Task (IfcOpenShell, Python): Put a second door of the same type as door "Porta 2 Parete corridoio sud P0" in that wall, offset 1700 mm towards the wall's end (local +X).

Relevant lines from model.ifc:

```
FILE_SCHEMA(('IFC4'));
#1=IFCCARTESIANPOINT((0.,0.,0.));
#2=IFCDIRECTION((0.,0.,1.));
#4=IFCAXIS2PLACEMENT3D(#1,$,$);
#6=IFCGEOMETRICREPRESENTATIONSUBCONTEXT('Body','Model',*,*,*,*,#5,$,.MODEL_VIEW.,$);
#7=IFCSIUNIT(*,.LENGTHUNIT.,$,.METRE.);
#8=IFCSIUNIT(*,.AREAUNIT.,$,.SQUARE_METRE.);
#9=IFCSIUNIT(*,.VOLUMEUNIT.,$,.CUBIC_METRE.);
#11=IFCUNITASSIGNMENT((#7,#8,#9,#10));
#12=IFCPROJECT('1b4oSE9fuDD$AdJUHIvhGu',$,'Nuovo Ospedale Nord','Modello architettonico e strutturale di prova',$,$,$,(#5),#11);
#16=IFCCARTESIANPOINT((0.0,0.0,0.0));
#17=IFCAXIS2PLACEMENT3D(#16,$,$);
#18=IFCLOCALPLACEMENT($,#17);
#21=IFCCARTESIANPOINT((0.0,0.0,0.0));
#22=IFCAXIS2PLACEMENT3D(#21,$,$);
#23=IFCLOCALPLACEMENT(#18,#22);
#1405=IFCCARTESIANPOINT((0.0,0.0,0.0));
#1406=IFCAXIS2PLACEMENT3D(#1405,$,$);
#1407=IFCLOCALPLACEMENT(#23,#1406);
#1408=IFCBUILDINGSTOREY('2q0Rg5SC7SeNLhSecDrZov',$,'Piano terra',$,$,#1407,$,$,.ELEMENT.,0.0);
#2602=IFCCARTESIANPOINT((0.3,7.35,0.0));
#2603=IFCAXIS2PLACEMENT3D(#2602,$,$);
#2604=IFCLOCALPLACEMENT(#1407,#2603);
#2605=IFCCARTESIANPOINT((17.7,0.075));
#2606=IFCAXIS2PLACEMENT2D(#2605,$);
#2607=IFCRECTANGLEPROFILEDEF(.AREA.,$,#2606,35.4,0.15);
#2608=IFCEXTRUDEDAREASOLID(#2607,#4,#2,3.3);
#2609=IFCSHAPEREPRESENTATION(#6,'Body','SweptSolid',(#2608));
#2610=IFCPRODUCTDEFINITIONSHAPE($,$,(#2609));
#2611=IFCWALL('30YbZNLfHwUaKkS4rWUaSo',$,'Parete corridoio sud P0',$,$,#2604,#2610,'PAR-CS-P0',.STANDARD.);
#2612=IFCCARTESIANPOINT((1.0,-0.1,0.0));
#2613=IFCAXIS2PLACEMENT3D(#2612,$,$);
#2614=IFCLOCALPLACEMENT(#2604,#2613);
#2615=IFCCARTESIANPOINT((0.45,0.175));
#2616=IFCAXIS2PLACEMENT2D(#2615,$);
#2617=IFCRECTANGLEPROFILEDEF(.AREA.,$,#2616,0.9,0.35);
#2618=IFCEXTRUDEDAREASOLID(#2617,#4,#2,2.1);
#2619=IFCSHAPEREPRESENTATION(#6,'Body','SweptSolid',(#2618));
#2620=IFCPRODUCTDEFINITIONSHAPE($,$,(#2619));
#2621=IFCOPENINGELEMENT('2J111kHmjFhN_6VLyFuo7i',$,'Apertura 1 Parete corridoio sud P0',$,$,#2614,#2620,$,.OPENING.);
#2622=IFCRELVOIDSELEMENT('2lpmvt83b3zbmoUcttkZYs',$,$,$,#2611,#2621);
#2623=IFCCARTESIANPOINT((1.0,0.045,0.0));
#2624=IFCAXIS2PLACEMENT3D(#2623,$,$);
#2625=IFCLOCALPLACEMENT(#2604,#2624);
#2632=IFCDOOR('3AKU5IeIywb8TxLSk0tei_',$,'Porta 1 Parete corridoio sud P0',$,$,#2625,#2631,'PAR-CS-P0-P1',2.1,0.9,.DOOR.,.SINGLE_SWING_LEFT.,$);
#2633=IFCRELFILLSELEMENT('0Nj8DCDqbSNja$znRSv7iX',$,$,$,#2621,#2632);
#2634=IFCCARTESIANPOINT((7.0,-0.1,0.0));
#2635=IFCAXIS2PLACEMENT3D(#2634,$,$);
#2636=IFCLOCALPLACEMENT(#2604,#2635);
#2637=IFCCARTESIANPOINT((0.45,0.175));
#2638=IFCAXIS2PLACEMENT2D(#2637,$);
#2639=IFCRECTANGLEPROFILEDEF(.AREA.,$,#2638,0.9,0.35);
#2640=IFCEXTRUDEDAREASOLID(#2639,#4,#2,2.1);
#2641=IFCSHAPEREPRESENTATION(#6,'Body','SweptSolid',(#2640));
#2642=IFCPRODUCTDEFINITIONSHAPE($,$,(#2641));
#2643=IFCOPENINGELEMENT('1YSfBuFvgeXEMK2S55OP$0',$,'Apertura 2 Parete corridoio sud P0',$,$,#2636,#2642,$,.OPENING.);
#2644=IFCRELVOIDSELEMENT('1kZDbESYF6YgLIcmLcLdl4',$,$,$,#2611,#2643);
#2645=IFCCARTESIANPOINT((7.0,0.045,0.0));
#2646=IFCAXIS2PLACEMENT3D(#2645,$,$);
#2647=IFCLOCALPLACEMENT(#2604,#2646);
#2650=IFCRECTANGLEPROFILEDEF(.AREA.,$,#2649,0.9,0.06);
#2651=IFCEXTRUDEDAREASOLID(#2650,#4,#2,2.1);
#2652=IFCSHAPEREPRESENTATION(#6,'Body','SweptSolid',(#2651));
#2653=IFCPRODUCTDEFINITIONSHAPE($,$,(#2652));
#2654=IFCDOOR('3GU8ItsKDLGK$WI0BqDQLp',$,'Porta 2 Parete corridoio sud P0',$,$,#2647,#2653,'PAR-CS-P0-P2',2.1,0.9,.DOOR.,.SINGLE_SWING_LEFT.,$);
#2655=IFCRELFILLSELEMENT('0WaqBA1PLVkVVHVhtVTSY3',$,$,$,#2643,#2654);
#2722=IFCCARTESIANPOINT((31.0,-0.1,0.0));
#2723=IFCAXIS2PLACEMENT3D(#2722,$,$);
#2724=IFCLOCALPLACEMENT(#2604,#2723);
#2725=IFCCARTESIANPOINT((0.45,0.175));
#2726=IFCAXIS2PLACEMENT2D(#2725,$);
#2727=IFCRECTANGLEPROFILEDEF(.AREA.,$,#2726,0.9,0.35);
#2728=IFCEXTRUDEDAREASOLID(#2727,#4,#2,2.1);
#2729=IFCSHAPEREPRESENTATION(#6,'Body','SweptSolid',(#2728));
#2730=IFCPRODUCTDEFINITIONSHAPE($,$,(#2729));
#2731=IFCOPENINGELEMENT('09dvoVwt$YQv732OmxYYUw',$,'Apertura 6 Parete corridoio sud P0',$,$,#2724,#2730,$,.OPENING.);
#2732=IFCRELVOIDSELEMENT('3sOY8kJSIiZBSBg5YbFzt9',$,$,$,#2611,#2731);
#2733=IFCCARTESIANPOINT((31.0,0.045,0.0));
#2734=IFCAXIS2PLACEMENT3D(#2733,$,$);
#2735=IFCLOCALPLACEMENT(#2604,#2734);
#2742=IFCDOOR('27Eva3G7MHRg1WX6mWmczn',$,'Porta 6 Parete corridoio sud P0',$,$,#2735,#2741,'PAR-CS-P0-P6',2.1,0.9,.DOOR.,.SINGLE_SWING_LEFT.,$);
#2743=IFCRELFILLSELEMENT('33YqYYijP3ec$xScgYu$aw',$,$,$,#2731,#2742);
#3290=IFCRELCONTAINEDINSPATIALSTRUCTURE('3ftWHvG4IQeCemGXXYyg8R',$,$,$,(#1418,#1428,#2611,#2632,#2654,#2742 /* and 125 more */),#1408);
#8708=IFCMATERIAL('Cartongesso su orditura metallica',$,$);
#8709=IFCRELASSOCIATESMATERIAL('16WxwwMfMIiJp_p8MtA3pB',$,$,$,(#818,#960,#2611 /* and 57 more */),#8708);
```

```python
import ifcopenshell
import ifcopenshell.api.feature
import ifcopenshell.api.geometry
import ifcopenshell.api.root
import ifcopenshell.geom
import ifcopenshell.util.element
import ifcopenshell.util.placement
import ifcopenshell.util.shape
import ifcopenshell.util.unit

model = ifcopenshell.open("model.ifc")
unit_scale = ifcopenshell.util.unit.calculate_unit_scale(model)
settings = ifcopenshell.geom.settings()


def volume(element):
    """Net volume in cubic metres, openings subtracted."""
    shape = ifcopenshell.geom.create_shape(settings, element)
    return ifcopenshell.util.shape.get_volume(shape.geometry)


door = model.by_id(2654)
opening = door.FillsVoids[0].RelatingOpeningElement
wall = opening.VoidsElements[0].RelatingBuildingElement
before = volume(wall)
shift = ifcopenshell.util.placement.get_local_placement(wall.ObjectPlacement)[:3, 0] * 1.7 / unit_scale

# copy_class copies the void relationship, type, container and properties, but no geometry.
new_opening = ifcopenshell.api.root.copy_class(model, product=opening)
new_opening.Representation = ifcopenshell.util.element.copy_deep(
    model, opening.Representation, exclude=["IfcGeometricRepresentationContext", "IfcRepresentationMap"]
)
new_door = ifcopenshell.api.root.copy_class(model, product=door)
new_door.Representation = ifcopenshell.util.element.copy_deep(
    model, door.Representation, exclude=["IfcGeometricRepresentationContext", "IfcRepresentationMap"]
)
new_door.Tag = None
ifcopenshell.api.feature.add_filling(model, opening=new_opening, element=new_door)

for old, new in ((opening, new_opening), (door, new_door)):
    matrix = ifcopenshell.util.placement.get_local_placement(old.ObjectPlacement)
    matrix[:3, 3] += shift
    ifcopenshell.api.geometry.edit_object_placement(model, product=new, matrix=matrix, is_si=False)

after = volume(wall)

print(f"wall volume {before:.3f} -> {after:.3f} m3")

model.write("model-out.ifc")
```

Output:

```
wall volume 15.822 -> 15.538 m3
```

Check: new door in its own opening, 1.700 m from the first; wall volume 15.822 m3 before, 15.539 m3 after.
